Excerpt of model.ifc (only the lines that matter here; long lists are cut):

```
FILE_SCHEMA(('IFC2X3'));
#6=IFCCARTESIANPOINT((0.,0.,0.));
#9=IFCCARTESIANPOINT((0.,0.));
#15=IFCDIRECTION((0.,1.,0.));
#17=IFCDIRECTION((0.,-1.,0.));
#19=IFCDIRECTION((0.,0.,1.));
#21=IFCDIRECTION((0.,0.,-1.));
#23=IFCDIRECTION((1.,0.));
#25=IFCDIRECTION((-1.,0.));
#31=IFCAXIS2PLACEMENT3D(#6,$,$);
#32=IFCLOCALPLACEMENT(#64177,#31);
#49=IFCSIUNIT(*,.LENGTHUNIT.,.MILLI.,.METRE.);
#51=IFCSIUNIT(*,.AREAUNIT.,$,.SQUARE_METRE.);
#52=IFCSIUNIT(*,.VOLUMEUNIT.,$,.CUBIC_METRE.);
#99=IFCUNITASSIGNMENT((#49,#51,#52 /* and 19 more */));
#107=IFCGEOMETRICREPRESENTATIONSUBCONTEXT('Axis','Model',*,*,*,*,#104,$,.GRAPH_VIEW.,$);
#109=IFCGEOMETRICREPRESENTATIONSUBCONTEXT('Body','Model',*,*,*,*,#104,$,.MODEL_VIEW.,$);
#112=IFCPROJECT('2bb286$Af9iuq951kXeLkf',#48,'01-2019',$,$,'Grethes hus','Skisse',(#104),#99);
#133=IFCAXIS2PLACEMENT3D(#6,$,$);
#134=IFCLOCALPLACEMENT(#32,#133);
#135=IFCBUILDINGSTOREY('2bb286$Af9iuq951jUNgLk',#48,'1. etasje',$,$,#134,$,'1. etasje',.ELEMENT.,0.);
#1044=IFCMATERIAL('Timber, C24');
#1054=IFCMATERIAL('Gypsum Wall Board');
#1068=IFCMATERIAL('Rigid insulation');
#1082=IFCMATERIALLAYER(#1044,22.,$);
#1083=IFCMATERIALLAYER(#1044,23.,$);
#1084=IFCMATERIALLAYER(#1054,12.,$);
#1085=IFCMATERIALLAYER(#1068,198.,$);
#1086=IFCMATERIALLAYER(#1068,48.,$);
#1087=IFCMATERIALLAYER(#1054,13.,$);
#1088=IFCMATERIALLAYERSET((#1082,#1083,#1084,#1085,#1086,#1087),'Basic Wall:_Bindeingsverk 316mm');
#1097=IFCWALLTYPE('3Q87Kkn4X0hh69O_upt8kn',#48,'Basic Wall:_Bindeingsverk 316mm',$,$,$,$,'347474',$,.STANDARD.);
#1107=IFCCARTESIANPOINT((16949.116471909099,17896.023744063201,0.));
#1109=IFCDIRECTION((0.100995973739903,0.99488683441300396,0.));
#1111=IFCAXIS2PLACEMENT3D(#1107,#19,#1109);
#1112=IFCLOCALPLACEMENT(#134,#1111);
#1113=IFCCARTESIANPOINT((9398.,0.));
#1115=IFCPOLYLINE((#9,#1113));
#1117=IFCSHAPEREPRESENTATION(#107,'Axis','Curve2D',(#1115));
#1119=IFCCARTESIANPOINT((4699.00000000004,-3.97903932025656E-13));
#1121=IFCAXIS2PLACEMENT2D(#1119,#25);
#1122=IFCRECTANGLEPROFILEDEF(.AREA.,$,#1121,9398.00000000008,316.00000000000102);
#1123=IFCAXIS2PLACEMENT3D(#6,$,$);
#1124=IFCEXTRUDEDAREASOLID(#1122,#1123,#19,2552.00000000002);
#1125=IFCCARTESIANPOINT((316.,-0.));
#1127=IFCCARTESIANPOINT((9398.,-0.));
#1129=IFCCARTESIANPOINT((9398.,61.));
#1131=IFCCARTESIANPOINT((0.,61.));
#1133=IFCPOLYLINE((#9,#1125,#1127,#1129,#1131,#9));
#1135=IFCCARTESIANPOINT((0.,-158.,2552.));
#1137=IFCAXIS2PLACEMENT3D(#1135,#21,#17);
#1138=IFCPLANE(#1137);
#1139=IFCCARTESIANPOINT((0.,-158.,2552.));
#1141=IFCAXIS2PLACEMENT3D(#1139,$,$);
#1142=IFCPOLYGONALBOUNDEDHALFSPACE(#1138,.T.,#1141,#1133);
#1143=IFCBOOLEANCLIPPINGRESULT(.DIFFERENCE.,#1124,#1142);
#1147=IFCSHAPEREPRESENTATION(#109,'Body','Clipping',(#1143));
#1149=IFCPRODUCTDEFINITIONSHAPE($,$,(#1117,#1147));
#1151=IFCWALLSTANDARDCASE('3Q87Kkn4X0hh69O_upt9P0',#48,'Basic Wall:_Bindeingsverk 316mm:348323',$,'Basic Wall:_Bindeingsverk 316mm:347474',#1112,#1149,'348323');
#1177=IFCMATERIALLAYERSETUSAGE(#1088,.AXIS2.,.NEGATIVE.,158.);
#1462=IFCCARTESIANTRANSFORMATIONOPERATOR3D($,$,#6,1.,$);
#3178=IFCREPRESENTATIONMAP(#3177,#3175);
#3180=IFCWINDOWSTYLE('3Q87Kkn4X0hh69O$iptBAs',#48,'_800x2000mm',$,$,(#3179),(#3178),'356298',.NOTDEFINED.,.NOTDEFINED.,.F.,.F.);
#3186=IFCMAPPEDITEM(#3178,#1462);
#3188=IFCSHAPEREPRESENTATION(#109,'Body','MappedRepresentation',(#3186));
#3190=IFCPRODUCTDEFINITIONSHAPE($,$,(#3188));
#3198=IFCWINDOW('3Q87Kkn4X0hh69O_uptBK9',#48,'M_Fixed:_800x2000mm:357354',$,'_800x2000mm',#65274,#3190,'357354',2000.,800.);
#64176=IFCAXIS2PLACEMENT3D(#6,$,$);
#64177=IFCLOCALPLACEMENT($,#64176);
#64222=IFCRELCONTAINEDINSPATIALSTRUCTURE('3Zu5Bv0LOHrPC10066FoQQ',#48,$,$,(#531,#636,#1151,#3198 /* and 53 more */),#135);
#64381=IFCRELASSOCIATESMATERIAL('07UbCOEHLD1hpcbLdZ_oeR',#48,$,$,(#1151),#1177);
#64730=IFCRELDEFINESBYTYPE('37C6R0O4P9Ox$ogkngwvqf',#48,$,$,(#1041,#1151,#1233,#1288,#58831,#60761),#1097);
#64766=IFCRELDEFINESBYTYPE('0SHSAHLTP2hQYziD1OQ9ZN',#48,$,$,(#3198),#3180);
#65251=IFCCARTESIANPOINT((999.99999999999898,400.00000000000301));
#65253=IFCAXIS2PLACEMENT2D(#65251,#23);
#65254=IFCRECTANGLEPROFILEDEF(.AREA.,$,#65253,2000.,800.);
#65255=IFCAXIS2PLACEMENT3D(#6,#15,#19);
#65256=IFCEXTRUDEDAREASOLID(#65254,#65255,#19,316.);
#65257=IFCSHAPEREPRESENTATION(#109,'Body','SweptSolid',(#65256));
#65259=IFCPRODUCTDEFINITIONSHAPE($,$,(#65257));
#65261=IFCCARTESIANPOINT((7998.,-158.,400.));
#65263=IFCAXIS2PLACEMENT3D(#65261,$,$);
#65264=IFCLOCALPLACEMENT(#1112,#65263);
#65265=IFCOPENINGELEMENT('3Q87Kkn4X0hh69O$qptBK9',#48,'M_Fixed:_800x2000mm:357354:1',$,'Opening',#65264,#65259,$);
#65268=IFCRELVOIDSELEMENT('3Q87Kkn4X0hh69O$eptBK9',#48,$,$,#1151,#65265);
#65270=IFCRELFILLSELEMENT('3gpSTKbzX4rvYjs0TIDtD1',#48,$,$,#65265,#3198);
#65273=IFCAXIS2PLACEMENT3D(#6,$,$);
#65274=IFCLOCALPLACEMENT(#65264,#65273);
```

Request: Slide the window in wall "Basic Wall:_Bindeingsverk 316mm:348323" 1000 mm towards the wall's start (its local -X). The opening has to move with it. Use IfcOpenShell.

```python
import ifcopenshell
import ifcopenshell.api.geometry
import ifcopenshell.util.placement

model = ifcopenshell.open("model.ifc")

window = model.by_guid("3Q87Kkn4X0hh69O_uptBK9")
opening = window.FillsVoids[0].RelatingOpeningElement
wall = opening.VoidsElements[0].RelatingBuildingElement

wall_matrix = ifcopenshell.util.placement.get_local_placement(wall.ObjectPlacement)
shift = wall_matrix[:3, 0] * -1000.0
before = ifcopenshell.util.placement.get_local_placement(window.ObjectPlacement)[:3, 3].copy()

# The window is placed relative to its opening, so it follows when the opening moves.
matrix = ifcopenshell.util.placement.get_local_placement(opening.ObjectPlacement)
matrix[:3, 3] += shift
ifcopenshell.api.geometry.edit_object_placement(
    model, product=opening, matrix=matrix, is_si=False, should_transform_children=True
)

after = ifcopenshell.util.placement.get_local_placement(window.ObjectPlacement)[:3, 3]
print("window moved by", (after - before).round(3) + 0.0)

model.write("model_rev.ifc")
```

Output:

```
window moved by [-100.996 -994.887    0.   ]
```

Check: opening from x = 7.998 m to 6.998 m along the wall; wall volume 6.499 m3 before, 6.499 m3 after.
